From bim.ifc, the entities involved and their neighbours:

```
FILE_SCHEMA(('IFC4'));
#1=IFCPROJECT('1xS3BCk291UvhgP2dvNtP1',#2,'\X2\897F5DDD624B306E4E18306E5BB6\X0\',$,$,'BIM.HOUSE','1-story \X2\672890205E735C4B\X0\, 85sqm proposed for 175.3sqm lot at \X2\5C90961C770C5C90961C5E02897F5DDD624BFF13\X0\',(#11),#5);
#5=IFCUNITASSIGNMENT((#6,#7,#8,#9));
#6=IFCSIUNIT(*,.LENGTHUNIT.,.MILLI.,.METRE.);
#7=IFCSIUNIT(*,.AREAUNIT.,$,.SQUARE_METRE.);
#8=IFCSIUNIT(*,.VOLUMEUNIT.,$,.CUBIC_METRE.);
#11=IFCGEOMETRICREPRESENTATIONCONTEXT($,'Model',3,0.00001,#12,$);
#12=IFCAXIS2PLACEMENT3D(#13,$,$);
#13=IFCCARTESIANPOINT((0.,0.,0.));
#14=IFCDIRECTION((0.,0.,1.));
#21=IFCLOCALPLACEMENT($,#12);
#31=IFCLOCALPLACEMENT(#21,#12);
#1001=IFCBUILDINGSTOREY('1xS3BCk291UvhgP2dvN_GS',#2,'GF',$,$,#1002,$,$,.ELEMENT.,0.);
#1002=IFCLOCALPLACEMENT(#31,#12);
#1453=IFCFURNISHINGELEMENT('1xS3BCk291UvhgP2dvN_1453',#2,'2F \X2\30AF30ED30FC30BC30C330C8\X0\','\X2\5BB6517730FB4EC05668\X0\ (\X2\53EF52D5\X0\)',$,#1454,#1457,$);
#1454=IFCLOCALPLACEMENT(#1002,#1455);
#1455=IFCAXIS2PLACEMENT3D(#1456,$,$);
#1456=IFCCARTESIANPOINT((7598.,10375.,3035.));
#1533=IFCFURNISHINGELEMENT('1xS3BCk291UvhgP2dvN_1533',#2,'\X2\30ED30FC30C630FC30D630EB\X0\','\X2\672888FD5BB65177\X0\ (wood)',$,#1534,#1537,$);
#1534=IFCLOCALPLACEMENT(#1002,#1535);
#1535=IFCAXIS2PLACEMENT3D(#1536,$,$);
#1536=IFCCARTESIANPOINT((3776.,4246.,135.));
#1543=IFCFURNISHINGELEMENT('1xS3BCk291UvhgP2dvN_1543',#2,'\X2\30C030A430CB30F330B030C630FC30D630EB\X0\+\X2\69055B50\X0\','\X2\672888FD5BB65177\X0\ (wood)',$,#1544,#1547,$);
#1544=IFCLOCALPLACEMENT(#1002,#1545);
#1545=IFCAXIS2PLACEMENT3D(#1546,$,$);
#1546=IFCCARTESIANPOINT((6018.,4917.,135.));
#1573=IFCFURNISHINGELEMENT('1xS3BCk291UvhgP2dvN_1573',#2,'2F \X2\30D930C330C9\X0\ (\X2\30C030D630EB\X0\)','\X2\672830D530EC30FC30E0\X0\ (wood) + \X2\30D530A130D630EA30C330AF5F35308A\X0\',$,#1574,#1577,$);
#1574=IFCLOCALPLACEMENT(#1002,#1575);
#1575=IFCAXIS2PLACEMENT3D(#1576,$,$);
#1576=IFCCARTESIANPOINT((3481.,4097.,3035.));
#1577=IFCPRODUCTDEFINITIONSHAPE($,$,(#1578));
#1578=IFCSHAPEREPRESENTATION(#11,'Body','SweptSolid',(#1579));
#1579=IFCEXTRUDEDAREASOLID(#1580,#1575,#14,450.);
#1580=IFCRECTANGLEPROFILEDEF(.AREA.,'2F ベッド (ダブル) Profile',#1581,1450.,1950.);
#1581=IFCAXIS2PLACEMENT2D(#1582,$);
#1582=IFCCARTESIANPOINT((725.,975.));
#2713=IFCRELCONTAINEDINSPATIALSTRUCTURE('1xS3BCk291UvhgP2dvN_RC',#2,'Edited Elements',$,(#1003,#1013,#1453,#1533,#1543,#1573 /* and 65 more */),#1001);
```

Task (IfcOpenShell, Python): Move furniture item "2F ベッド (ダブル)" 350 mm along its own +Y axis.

```python
import ifcopenshell
import ifcopenshell.api.geometry
import ifcopenshell.util.placement
import ifcopenshell.util.unit

model = ifcopenshell.open("bim.ifc")
unit_scale = ifcopenshell.util.unit.calculate_unit_scale(model)

item = model.by_guid("1xS3BCk291UvhgP2dvN_1573")
matrix = ifcopenshell.util.placement.get_local_placement(item.ObjectPlacement)
matrix[:3, 3] += matrix[:3, 1] * 0.35 / unit_scale
ifcopenshell.api.geometry.edit_object_placement(model, product=item, matrix=matrix, is_si=False)

print(ifcopenshell.util.placement.get_local_placement(item.ObjectPlacement).round(3) + 0.0)

model.write("bim_updated.ifc")
```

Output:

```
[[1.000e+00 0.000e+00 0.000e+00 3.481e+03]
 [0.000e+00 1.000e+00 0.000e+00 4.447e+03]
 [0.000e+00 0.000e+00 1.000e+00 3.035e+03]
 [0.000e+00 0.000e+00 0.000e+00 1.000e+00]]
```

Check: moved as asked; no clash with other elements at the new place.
